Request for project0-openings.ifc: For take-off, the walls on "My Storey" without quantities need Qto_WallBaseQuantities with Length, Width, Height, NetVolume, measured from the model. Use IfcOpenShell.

First a look at what the model holds.

```python
import ifcopenshell
import ifcopenshell.util.element
import ifcopenshell.util.unit

model = ifcopenshell.open("project0-openings.ifc")
print(model.schema)
for unit_type in ("LENGTHUNIT", "AREAUNIT", "VOLUMEUNIT"):
    print(unit_type, ifcopenshell.util.unit.calculate_unit_scale(model, unit_type))
storey = next(s for s in model.by_type("IfcBuildingStorey") if s.Name == "My Storey")
walls = [e for e in ifcopenshell.util.element.get_decomposition(storey) if e.is_a("IfcWall")]
for e in sorted(walls, key=lambda e: e.id()):
    print(e.id(), e.is_a(), e.Name, list(ifcopenshell.util.element.get_psets(e, qtos_only=True)), sep=" | ")
```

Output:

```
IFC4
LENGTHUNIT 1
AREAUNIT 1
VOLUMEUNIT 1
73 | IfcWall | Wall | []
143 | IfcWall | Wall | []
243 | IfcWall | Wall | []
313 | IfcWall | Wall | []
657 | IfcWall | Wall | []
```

```python
import ifcopenshell
import ifcopenshell.api.pset
import ifcopenshell.geom
import ifcopenshell.util.element
import ifcopenshell.util.shape
import ifcopenshell.util.unit

model = ifcopenshell.open("project0-openings.ifc")
unit_scale = ifcopenshell.util.unit.calculate_unit_scale(model)
volume_scale = ifcopenshell.util.unit.calculate_unit_scale(model, "VOLUMEUNIT")
settings = ifcopenshell.geom.settings()

storey = next(s for s in model.by_type("IfcBuildingStorey") if s.Name == "My Storey")
walls = [e for e in ifcopenshell.util.element.get_decomposition(storey) if e.is_a("IfcWall")]

for e in sorted(walls, key=lambda e: e.id()):
    if ifcopenshell.util.element.get_psets(e, qtos_only=True, should_inherit=False):
        continue
    # Geometry comes back in metres, in the element's own axes.
    shape = ifcopenshell.geom.create_shape(settings, e)
    values = {
        "Length": ifcopenshell.util.shape.get_x(shape.geometry) / unit_scale,
        "Width": ifcopenshell.util.shape.get_y(shape.geometry) / unit_scale,
        "Height": ifcopenshell.util.shape.get_z(shape.geometry) / unit_scale,
        "NetVolume": ifcopenshell.util.shape.get_volume(shape.geometry) / volume_scale,
    }
    qto = ifcopenshell.api.pset.add_qto(model, product=e, name="Qto_WallBaseQuantities")
    ifcopenshell.api.pset.edit_qto(model, qto=qto, properties=values)
    print(e.id(), {k: round(v, 3) for k, v in values.items()})

model.write("project0-openings_updated.ifc")
```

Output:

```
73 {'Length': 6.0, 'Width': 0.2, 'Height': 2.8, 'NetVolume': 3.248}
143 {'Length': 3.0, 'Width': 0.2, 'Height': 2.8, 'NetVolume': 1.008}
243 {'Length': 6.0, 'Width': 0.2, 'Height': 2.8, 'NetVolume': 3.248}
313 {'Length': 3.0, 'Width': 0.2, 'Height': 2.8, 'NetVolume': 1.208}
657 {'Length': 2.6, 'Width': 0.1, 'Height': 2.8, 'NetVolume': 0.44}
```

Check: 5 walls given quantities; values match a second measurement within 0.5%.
